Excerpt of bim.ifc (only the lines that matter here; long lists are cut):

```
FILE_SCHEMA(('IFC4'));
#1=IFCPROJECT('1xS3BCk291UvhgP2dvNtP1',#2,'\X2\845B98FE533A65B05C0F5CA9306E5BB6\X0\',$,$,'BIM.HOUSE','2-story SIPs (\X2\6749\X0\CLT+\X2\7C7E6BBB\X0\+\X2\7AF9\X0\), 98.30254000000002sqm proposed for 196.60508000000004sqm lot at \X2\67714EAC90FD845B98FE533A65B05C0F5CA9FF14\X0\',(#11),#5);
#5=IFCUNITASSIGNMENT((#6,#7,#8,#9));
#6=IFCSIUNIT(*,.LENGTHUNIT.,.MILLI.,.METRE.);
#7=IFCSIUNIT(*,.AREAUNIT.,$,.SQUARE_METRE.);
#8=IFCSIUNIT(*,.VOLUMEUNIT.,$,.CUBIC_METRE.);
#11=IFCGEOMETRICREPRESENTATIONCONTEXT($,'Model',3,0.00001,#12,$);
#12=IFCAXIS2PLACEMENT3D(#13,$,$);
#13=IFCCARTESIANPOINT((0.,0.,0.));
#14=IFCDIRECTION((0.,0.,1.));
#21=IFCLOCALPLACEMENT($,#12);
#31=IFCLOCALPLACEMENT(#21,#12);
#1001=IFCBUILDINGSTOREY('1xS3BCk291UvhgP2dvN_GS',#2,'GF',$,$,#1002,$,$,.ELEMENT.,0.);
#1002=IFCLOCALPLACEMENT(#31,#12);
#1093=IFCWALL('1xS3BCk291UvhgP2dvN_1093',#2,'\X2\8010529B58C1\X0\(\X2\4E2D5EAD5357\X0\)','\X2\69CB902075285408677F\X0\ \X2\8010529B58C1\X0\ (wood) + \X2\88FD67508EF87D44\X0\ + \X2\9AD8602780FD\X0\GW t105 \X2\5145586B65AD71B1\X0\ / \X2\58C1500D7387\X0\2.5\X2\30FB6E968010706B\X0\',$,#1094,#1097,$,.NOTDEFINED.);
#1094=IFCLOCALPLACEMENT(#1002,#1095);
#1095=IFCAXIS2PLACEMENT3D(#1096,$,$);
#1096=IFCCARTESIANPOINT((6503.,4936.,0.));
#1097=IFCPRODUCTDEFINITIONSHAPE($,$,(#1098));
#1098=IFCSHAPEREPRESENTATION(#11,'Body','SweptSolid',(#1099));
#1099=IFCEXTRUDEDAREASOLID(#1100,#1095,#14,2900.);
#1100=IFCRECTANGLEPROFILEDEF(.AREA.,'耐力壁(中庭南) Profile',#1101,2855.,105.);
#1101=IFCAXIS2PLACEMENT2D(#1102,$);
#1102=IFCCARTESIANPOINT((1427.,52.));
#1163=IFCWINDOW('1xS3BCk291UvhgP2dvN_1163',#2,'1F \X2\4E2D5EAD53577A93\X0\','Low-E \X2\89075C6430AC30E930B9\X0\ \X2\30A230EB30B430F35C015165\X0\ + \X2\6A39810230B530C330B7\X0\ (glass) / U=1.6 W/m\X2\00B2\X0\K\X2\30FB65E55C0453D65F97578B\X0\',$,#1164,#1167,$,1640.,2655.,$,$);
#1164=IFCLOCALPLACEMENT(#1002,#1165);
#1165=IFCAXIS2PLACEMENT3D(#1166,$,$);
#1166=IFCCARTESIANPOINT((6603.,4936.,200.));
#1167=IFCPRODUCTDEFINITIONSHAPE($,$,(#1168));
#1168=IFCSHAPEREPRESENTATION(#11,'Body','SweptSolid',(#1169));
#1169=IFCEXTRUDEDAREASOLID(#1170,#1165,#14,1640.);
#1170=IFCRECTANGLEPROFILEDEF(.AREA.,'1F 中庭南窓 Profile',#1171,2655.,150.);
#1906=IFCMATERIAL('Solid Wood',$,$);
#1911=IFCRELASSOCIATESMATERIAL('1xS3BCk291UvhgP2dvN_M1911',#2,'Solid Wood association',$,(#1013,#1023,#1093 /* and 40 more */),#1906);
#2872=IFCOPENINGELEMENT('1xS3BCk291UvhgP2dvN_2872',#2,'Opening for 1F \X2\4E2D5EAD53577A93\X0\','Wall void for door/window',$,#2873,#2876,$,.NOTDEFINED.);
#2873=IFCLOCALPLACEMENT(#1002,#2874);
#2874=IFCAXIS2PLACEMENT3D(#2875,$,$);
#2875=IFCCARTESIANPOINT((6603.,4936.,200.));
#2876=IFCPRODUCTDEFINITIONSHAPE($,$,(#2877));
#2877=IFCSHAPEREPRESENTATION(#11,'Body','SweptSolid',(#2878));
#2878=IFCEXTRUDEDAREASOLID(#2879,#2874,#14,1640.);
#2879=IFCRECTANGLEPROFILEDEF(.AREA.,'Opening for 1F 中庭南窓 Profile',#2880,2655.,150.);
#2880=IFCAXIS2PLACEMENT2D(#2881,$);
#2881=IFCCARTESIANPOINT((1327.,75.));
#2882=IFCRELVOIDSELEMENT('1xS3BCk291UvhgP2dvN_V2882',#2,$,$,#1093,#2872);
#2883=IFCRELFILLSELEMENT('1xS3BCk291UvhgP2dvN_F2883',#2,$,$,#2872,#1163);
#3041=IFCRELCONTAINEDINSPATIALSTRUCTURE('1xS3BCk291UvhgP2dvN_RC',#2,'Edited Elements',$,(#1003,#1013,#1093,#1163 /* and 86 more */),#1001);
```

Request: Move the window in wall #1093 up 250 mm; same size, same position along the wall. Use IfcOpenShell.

```python
import numpy as np
import ifcopenshell
import ifcopenshell.api.geometry
import ifcopenshell.util.placement
import ifcopenshell.util.unit

model = ifcopenshell.open("bim.ifc")
unit_scale = ifcopenshell.util.unit.calculate_unit_scale(model)

window = model.by_id(1163)
opening = window.FillsVoids[0].RelatingOpeningElement
dz = 250.0

shift = np.array([0.0, 0.0, dz])
# The window is not placed relative to its opening, so move both.
for product in (opening, window):
    matrix = ifcopenshell.util.placement.get_local_placement(product.ObjectPlacement)
    matrix[:3, 3] += shift
    ifcopenshell.api.geometry.edit_object_placement(model, product=product, matrix=matrix, is_si=False)

print(f"moved by {dz * unit_scale:+.3f} m")

model.write("bim-out.ifc")
```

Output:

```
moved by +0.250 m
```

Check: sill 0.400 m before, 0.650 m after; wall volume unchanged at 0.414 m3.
